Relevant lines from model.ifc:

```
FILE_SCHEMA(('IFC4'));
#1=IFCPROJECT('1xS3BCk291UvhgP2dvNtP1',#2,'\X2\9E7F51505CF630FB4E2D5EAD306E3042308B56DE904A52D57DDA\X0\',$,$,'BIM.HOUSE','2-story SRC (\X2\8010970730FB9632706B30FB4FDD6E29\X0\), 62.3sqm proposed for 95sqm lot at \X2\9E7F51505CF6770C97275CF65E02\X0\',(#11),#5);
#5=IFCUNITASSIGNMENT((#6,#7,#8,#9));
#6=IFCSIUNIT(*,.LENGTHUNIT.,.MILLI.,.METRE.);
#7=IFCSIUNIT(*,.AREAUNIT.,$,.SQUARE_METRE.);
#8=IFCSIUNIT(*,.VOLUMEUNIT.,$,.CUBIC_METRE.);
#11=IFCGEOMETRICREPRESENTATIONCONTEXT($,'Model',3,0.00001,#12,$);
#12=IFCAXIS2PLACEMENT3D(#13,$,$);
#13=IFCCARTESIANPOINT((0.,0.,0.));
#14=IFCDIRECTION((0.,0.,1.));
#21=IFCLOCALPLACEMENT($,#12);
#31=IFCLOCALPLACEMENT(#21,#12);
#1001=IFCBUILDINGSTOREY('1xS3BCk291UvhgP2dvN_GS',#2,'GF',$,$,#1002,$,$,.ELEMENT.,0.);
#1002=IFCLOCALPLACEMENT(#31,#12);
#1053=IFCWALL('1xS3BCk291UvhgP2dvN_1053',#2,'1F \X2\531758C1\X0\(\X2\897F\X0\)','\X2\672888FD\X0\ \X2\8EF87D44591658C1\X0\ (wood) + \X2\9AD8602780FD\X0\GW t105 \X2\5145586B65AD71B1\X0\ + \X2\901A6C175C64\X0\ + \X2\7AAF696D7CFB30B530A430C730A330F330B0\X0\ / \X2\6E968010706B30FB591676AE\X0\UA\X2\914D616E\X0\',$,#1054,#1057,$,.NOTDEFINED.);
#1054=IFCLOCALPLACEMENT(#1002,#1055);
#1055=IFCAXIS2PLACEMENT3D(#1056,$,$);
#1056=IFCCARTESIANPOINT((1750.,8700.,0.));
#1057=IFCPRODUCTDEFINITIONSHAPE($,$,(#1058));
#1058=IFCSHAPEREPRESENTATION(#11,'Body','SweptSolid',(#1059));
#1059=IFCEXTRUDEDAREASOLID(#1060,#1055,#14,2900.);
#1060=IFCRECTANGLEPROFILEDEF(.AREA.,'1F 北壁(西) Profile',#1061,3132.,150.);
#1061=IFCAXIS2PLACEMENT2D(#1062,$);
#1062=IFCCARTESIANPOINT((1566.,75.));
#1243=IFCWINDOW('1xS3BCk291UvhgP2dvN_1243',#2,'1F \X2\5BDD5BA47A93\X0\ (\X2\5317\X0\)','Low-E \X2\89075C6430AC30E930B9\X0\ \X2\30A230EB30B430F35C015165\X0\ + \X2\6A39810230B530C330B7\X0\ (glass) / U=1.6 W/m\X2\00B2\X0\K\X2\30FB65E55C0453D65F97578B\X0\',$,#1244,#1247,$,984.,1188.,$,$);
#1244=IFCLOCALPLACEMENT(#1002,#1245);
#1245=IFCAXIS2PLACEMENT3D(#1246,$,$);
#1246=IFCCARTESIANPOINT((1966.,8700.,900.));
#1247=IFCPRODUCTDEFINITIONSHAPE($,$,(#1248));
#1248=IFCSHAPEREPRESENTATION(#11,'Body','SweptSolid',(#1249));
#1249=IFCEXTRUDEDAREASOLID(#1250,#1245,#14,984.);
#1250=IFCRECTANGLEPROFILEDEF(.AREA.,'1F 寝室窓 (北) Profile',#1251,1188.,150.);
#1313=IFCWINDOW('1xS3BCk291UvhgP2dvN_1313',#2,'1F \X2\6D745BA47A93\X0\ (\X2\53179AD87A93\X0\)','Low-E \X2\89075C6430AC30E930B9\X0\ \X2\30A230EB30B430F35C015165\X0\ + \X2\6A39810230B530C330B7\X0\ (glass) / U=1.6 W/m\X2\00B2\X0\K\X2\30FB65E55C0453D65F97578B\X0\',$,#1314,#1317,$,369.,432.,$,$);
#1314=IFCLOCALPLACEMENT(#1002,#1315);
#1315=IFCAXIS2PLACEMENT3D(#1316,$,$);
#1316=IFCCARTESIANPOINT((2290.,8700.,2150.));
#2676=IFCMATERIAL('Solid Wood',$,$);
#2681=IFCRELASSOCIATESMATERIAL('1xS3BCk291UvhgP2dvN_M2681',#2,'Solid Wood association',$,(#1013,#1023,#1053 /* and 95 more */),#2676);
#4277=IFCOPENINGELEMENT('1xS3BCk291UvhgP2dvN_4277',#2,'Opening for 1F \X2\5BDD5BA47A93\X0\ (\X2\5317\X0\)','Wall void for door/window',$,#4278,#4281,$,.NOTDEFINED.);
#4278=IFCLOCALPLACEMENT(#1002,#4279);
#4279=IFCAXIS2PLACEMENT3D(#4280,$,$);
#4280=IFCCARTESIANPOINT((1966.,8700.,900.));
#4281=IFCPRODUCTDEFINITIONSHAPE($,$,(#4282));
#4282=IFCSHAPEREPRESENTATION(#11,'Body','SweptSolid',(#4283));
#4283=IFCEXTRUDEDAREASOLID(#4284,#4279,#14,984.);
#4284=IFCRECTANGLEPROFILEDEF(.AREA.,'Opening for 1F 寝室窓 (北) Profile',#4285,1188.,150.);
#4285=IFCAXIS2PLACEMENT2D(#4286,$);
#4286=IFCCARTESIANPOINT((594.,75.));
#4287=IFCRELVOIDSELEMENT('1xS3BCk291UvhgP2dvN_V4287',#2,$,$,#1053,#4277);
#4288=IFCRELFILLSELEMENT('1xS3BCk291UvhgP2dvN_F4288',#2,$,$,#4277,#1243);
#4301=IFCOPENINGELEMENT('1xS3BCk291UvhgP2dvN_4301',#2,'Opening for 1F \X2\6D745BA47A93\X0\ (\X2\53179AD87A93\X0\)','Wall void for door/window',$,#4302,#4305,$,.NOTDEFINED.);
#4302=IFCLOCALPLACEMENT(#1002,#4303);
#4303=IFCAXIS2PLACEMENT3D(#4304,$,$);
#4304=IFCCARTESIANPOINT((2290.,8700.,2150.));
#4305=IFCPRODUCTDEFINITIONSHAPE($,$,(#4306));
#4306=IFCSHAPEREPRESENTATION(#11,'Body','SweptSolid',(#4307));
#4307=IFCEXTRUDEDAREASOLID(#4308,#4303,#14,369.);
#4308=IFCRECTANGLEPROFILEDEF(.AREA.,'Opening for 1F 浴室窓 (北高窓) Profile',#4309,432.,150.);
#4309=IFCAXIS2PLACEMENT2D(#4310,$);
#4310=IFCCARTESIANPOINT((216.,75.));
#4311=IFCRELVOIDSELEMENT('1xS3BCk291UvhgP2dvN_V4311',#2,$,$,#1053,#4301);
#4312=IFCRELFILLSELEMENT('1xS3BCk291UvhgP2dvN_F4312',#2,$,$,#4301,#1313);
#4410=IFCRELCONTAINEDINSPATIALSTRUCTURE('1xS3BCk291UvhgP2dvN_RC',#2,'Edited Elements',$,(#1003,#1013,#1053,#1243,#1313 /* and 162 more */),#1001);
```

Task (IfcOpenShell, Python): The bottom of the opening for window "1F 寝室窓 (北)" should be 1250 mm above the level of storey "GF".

```python
import numpy as np
import ifcopenshell
import ifcopenshell.api.geometry
import ifcopenshell.geom
import ifcopenshell.util.element
import ifcopenshell.util.placement
import ifcopenshell.util.shape
import ifcopenshell.util.unit

model = ifcopenshell.open("model.ifc")
unit_scale = ifcopenshell.util.unit.calculate_unit_scale(model)

window = model.by_guid("1xS3BCk291UvhgP2dvN_1243")
opening = window.FillsVoids[0].RelatingOpeningElement
storey = ifcopenshell.util.element.get_container(window, ifc_class="IfcBuildingStorey")
level = ifcopenshell.util.placement.get_local_placement(storey.ObjectPlacement)[2, 3]

# The opening's origin need not be at the sill, so measure its lowest point.
shape = ifcopenshell.geom.create_shape(ifcopenshell.geom.settings(), opening)
bottom = ifcopenshell.util.shape.get_shape_bottom_elevation(shape, shape.geometry) / unit_scale
dz = level + 1.25 / unit_scale - bottom

shift = np.array([0.0, 0.0, dz])
# The window is not placed relative to its opening, so move both.
for product in (opening, window):
    matrix = ifcopenshell.util.placement.get_local_placement(product.ObjectPlacement)
    matrix[:3, 3] += shift
    ifcopenshell.api.geometry.edit_object_placement(model, product=product, matrix=matrix, is_si=False)

print(f"moved by {dz * unit_scale:+.3f} m")

model.write("model-out.ifc")
```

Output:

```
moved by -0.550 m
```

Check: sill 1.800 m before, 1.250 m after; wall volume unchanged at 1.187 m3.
